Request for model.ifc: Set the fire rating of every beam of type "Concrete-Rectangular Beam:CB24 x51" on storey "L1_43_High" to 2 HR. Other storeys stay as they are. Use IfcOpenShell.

First a look at what the model holds.

```python
import ifcopenshell
import ifcopenshell.util.element

model = ifcopenshell.open("model.ifc")
print(model.schema)
storey = next(s for s in model.by_type("IfcBuildingStorey") if s.Name == "L1_43_High")
beams = [e for e in ifcopenshell.util.element.get_decomposition(storey) if e.is_a("IfcBeam")]
seen = {}
for e in beams:
    element_type = ifcopenshell.util.element.get_type(e)
    key = (element_type.Name if element_type != e and element_type else None, ifcopenshell.util.element.get_pset(e, "Pset_BeamCommon", "FireRating"))
    seen[key] = seen.get(key, 0) + 1
for (name, value), count in sorted(seen.items(), key=str):
    print(count, "x", name, "|", value)
```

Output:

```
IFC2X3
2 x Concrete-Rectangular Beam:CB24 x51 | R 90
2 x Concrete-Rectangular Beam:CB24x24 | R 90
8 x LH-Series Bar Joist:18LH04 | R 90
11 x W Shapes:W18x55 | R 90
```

```python
import ifcopenshell
import ifcopenshell.api.pset
import ifcopenshell.util.element

model = ifcopenshell.open("model.ifc")

storey = next(s for s in model.by_type("IfcBuildingStorey") if s.Name == "L1_43_High")
beams = [e for e in ifcopenshell.util.element.get_decomposition(storey) if e.is_a("IfcBeam")]

count = 0
for e in beams:
    element_type = ifcopenshell.util.element.get_type(e)
    if element_type in (None, e) or element_type.Name != "Concrete-Rectangular Beam:CB24 x51":
        continue
    # add_pset returns the element's existing set when there is one.
    pset = ifcopenshell.api.pset.add_pset(model, product=e, name="Pset_BeamCommon")
    ifcopenshell.api.pset.edit_pset(model, pset=pset, properties={"FireRating": "2 HR"})
    count += 1

print(count, "beams updated")

model.write("model_rev.ifc")
```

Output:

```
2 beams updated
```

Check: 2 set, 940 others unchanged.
